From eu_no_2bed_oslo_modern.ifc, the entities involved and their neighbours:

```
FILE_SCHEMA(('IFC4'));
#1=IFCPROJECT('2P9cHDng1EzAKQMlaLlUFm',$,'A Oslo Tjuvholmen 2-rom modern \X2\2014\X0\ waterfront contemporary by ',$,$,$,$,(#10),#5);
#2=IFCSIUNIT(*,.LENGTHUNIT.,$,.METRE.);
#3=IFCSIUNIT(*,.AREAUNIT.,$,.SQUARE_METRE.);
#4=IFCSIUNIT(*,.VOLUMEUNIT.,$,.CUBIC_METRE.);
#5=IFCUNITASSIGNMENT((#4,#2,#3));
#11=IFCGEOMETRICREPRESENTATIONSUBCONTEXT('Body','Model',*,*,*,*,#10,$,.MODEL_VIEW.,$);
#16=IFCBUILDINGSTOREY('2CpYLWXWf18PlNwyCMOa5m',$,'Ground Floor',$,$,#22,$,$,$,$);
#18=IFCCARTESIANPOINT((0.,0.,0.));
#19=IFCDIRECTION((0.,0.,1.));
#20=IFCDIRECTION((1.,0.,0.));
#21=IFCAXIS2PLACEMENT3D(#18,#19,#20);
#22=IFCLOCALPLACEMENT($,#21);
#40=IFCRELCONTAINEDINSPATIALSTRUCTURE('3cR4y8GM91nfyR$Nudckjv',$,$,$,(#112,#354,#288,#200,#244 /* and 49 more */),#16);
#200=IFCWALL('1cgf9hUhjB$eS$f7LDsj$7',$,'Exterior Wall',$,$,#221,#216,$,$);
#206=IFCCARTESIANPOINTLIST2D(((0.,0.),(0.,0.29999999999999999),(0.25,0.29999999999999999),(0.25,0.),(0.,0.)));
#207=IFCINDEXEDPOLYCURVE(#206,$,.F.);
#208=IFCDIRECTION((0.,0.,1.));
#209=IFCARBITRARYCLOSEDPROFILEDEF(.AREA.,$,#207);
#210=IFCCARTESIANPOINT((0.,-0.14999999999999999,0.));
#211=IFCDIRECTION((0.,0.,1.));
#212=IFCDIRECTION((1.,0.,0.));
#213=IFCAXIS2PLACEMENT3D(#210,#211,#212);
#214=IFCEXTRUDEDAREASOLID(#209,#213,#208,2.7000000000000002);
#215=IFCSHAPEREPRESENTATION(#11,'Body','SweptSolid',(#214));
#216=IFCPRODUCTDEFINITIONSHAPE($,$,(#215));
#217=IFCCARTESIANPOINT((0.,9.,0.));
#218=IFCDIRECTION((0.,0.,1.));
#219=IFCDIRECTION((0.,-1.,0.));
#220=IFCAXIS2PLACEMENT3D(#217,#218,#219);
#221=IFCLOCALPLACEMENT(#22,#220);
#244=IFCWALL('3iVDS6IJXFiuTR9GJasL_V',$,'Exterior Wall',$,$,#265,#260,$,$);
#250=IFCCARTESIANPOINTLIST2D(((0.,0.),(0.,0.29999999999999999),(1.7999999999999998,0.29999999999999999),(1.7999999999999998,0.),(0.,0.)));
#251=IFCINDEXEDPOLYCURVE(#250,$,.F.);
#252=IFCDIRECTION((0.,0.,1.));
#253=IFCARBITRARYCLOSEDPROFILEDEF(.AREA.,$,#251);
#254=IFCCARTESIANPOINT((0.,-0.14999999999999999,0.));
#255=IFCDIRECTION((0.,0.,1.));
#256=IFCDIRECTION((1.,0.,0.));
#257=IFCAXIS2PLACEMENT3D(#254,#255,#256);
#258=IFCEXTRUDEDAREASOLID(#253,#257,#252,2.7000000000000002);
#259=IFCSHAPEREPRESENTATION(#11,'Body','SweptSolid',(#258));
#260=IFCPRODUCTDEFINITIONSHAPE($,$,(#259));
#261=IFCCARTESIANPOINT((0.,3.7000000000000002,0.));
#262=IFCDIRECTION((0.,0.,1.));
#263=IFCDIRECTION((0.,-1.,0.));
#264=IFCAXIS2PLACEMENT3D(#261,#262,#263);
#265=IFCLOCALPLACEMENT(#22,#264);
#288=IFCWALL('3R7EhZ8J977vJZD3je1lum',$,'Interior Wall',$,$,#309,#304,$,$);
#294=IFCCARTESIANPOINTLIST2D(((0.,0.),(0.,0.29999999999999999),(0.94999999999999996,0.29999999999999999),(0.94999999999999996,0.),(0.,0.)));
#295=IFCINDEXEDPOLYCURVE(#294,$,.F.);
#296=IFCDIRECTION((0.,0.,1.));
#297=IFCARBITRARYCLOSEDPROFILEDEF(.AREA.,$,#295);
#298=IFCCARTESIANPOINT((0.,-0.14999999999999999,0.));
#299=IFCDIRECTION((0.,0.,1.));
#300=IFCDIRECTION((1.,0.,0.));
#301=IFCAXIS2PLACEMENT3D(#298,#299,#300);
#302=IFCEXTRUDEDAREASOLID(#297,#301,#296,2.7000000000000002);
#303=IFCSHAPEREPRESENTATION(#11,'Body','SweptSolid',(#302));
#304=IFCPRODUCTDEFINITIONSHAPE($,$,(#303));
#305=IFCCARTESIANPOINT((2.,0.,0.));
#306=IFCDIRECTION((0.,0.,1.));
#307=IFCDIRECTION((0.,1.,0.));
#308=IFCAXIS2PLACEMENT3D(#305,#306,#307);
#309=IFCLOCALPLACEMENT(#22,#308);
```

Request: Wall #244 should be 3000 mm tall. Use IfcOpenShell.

```python
import ifcopenshell
import ifcopenshell.geom
import ifcopenshell.util.representation
import ifcopenshell.util.shape

model = ifcopenshell.open("eu_no_2bed_oslo_modern.ifc")
settings = ifcopenshell.geom.settings()


def volume(element):
    """Net volume in cubic metres, openings subtracted."""
    shape = ifcopenshell.geom.create_shape(settings, element)
    return ifcopenshell.util.shape.get_volume(shape.geometry)


wall = model.by_id(244)
before = volume(wall)

body = ifcopenshell.util.representation.get_representation(wall, "Model", "Body")
solid = body.Items[0]
old_height = solid.Depth
solid.Depth = 3.0
after = volume(wall)

print(f"height {old_height:g} -> {solid.Depth:g}, volume {before:.3f} -> {after:.3f} m3")

model.write("eu_no_2bed_oslo_modern_updated.ifc")
```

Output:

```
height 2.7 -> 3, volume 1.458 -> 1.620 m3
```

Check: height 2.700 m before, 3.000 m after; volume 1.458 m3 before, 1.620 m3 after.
